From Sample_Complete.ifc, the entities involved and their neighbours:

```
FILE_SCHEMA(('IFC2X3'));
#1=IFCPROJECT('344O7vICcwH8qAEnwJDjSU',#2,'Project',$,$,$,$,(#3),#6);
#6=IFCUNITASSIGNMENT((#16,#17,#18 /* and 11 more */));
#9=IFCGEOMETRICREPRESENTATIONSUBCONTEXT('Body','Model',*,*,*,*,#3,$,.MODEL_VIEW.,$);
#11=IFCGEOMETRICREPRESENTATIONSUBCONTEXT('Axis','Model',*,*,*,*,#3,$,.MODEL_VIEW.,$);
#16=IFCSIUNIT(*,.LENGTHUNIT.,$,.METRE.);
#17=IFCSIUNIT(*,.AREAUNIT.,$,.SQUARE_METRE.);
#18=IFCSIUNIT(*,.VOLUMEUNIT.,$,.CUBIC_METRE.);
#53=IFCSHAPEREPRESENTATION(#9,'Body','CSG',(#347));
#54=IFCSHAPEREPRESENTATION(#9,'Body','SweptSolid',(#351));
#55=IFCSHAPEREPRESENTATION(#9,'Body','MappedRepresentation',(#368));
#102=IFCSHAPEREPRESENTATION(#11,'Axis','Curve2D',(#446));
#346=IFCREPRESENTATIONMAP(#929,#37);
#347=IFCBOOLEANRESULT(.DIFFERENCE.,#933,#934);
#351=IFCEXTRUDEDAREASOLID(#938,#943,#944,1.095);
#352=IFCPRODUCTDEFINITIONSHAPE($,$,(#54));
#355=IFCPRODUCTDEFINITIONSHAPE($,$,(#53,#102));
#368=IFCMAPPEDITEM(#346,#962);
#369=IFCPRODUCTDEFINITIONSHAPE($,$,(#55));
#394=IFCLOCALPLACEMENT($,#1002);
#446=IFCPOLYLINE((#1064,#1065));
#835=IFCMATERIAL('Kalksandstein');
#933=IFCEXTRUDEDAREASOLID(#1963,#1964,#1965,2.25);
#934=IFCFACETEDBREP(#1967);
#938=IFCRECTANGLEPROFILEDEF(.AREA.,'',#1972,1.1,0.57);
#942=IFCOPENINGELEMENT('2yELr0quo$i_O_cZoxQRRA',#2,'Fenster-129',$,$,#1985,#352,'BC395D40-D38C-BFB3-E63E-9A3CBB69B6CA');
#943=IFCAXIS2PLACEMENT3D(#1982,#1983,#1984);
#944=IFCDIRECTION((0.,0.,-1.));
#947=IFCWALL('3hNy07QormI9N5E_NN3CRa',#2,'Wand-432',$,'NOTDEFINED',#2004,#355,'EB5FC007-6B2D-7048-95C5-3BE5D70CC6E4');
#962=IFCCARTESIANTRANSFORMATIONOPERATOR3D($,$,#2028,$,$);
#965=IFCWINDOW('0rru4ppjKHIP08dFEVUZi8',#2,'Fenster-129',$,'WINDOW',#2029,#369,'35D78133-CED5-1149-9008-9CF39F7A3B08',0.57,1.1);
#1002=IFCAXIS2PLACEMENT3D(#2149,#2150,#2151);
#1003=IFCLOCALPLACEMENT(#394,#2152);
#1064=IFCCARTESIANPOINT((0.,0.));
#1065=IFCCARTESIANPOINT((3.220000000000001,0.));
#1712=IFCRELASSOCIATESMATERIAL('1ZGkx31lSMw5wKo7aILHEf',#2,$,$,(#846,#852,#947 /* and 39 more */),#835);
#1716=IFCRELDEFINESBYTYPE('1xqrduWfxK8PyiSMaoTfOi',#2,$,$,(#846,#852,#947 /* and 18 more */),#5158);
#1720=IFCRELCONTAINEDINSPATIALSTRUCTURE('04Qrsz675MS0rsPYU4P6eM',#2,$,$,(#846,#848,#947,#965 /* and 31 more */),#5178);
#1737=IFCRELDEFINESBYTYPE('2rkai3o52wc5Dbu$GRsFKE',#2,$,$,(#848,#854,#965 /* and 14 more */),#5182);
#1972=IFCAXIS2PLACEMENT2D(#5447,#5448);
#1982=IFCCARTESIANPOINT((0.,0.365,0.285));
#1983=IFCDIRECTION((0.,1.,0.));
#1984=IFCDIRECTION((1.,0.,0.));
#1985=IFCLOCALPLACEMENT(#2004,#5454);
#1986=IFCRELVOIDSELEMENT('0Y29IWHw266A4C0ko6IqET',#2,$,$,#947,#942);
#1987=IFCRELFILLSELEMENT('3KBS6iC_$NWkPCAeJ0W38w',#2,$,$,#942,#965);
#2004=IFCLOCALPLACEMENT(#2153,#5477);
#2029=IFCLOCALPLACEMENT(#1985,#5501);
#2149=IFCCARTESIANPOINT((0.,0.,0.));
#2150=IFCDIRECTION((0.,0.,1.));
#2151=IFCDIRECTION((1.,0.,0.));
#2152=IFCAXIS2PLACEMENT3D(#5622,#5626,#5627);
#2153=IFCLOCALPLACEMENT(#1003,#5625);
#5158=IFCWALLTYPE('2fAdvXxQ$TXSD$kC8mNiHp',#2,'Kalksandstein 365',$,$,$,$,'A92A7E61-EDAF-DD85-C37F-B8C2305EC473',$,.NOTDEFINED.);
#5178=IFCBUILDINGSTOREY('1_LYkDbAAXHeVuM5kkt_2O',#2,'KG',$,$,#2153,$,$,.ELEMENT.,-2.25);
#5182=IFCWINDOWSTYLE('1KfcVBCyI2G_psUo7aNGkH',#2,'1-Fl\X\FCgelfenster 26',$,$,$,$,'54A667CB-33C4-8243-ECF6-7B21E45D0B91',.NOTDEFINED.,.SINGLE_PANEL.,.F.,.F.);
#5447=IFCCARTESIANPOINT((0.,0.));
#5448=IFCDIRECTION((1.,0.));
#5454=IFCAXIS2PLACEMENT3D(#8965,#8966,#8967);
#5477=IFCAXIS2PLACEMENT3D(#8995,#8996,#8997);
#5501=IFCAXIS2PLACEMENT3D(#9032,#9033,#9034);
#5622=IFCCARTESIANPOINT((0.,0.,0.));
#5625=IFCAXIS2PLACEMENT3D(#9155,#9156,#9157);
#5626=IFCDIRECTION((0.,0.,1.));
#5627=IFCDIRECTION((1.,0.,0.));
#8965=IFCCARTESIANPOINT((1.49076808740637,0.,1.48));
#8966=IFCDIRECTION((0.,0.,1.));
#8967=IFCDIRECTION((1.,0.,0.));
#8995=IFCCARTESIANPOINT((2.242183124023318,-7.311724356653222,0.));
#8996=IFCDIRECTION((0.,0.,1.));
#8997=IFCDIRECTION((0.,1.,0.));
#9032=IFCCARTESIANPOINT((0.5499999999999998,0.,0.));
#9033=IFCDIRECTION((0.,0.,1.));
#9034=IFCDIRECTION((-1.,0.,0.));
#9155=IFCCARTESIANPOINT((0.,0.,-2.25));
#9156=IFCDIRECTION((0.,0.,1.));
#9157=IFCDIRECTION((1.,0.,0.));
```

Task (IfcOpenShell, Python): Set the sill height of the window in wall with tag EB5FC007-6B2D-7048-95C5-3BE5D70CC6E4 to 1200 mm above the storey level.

```python
import numpy as np
import ifcopenshell
import ifcopenshell.api.geometry
import ifcopenshell.geom
import ifcopenshell.util.element
import ifcopenshell.util.placement
import ifcopenshell.util.shape
import ifcopenshell.util.unit

model = ifcopenshell.open("Sample_Complete.ifc")
unit_scale = ifcopenshell.util.unit.calculate_unit_scale(model)

window = model.by_guid("0rru4ppjKHIP08dFEVUZi8")
opening = window.FillsVoids[0].RelatingOpeningElement
storey = ifcopenshell.util.element.get_container(window, ifc_class="IfcBuildingStorey")
level = ifcopenshell.util.placement.get_local_placement(storey.ObjectPlacement)[2, 3]

# The opening's origin need not be at the sill, so measure its lowest point.
shape = ifcopenshell.geom.create_shape(ifcopenshell.geom.settings(), opening)
bottom = ifcopenshell.util.shape.get_shape_bottom_elevation(shape, shape.geometry) / unit_scale
dz = level + 1.2 / unit_scale - bottom

shift = np.array([0.0, 0.0, dz])
# The window is placed relative to its opening, so it follows when the opening moves.
matrix = ifcopenshell.util.placement.get_local_placement(opening.ObjectPlacement)
matrix[:3, 3] += shift
ifcopenshell.api.geometry.edit_object_placement(
    model, product=opening, matrix=matrix, is_si=False, should_transform_children=True
)

print(f"moved by {dz * unit_scale:+.3f} m")

model.write("Sample_Complete_v2.ifc")
```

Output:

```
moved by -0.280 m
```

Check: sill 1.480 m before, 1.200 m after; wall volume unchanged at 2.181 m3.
